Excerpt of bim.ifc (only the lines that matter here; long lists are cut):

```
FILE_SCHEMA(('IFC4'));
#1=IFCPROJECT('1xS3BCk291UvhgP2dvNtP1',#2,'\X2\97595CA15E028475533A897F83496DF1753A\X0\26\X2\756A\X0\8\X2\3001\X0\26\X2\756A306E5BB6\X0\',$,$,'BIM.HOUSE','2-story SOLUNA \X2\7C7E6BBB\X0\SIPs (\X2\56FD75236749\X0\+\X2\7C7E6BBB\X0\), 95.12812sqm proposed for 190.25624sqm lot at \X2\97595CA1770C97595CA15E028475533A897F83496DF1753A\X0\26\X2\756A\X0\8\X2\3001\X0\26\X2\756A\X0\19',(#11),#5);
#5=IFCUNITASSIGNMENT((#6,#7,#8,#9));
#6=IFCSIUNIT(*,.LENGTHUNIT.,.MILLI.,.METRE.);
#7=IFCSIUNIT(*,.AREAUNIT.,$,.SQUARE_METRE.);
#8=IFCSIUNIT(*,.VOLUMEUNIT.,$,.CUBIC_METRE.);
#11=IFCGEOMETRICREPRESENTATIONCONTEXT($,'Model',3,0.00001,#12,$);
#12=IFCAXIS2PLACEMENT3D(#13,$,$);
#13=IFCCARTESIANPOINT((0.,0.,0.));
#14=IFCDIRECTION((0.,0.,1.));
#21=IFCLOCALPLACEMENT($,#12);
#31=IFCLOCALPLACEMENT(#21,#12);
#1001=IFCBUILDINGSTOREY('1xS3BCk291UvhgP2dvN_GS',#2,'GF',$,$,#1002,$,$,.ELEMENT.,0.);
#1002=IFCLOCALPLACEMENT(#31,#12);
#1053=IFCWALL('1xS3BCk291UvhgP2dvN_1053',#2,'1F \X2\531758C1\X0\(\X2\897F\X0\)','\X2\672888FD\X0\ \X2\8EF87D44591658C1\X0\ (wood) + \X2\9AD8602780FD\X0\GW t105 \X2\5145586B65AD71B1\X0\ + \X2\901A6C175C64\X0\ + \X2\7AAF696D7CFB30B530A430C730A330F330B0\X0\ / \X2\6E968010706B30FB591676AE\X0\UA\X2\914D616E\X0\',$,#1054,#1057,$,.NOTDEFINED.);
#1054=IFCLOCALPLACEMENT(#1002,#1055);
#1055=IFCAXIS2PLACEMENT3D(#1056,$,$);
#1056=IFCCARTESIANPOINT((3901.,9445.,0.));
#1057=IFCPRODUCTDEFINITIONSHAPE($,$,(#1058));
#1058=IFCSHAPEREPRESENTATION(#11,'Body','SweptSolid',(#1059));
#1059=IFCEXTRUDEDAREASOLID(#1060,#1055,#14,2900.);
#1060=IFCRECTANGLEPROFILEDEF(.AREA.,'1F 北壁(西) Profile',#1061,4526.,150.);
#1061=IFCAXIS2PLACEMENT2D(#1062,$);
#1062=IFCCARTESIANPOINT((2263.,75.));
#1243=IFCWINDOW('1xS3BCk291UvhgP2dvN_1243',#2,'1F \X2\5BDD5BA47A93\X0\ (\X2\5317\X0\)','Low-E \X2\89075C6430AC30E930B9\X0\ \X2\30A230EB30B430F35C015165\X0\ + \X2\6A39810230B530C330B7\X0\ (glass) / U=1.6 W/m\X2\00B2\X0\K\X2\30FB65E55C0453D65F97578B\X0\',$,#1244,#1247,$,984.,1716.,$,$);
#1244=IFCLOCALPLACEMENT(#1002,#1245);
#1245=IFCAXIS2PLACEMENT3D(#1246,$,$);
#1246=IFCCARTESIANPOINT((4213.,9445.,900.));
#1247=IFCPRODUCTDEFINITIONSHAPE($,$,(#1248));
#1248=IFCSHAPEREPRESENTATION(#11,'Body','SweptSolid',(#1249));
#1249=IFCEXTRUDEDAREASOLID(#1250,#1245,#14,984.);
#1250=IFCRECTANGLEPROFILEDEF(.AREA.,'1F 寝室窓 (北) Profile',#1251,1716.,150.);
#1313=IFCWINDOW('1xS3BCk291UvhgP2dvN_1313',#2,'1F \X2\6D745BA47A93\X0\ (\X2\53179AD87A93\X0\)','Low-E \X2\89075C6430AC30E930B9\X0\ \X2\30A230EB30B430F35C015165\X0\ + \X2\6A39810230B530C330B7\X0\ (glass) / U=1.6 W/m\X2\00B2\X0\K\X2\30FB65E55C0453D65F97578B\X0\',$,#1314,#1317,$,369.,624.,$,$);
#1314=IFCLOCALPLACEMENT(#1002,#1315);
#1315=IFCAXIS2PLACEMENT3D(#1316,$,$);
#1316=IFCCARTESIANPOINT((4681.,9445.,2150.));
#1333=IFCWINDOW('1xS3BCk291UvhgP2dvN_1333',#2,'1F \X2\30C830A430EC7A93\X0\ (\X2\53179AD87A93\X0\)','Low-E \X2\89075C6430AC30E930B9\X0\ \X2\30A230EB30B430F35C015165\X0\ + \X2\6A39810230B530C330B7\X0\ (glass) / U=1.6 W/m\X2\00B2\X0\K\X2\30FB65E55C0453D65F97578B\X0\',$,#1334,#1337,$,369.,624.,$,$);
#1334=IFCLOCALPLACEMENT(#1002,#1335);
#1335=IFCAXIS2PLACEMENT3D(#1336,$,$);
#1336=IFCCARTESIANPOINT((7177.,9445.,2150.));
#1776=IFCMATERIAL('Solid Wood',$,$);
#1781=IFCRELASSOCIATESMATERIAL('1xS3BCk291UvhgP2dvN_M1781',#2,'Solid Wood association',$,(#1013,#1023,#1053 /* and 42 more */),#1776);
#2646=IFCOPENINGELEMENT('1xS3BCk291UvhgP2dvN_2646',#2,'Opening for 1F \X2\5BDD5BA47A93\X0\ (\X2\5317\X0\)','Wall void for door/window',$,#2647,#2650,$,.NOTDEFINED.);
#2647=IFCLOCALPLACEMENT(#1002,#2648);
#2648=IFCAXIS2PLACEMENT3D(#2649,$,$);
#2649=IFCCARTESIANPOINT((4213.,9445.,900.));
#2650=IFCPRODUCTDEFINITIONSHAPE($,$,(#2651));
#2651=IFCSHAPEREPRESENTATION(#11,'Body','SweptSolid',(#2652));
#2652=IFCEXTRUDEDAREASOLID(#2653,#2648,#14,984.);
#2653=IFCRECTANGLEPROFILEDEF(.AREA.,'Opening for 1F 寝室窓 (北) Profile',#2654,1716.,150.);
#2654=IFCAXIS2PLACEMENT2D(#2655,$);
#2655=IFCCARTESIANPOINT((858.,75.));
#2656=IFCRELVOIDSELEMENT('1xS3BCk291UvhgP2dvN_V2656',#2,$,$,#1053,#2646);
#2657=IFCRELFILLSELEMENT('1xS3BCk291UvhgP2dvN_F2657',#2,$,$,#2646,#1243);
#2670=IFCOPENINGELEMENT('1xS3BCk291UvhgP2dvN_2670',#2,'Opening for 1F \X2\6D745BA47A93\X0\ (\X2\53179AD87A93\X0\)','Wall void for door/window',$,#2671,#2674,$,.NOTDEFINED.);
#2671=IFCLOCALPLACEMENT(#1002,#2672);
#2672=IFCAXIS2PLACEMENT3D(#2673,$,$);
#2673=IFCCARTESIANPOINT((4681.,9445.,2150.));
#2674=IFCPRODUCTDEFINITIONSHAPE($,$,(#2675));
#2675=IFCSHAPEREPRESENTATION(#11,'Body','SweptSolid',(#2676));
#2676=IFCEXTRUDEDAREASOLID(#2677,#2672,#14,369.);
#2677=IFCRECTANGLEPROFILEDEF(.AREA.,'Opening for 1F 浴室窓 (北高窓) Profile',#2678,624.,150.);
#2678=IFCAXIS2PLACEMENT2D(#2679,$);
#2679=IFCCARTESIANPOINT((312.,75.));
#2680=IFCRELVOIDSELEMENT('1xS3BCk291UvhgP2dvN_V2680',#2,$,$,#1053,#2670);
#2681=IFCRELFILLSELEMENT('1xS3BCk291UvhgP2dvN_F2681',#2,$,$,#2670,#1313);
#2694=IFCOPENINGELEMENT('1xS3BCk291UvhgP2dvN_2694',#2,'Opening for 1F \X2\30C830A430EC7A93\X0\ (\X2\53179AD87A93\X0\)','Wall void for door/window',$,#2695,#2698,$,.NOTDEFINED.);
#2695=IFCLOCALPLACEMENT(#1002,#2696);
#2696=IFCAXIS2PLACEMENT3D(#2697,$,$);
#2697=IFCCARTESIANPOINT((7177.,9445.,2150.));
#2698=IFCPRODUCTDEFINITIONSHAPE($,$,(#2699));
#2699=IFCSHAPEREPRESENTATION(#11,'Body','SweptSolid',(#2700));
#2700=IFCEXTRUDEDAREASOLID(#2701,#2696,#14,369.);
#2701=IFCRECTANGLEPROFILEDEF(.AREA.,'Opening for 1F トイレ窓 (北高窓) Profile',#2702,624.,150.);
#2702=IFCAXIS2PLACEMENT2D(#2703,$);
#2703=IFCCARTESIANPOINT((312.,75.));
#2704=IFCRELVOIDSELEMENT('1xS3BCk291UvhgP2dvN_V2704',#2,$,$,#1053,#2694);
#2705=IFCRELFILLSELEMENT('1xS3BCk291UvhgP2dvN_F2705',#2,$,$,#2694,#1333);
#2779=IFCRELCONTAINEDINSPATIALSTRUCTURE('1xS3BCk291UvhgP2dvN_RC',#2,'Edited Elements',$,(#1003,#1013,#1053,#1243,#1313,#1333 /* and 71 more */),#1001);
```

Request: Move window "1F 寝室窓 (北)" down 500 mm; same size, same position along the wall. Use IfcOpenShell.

```python
import numpy as np
import ifcopenshell
import ifcopenshell.api.geometry
import ifcopenshell.util.placement
import ifcopenshell.util.unit

model = ifcopenshell.open("bim.ifc")
unit_scale = ifcopenshell.util.unit.calculate_unit_scale(model)

window = model.by_guid("1xS3BCk291UvhgP2dvN_1243")
opening = window.FillsVoids[0].RelatingOpeningElement
dz = -500.0

shift = np.array([0.0, 0.0, dz])
# The window is not placed relative to its opening, so move both.
for product in (opening, window):
    matrix = ifcopenshell.util.placement.get_local_placement(product.ObjectPlacement)
    matrix[:3, 3] += shift
    ifcopenshell.api.geometry.edit_object_placement(model, product=product, matrix=matrix, is_si=False)

print(f"moved by {dz * unit_scale:+.3f} m")

model.write("bim_updated.ifc")
```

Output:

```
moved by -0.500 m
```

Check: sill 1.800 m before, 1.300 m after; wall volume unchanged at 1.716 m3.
